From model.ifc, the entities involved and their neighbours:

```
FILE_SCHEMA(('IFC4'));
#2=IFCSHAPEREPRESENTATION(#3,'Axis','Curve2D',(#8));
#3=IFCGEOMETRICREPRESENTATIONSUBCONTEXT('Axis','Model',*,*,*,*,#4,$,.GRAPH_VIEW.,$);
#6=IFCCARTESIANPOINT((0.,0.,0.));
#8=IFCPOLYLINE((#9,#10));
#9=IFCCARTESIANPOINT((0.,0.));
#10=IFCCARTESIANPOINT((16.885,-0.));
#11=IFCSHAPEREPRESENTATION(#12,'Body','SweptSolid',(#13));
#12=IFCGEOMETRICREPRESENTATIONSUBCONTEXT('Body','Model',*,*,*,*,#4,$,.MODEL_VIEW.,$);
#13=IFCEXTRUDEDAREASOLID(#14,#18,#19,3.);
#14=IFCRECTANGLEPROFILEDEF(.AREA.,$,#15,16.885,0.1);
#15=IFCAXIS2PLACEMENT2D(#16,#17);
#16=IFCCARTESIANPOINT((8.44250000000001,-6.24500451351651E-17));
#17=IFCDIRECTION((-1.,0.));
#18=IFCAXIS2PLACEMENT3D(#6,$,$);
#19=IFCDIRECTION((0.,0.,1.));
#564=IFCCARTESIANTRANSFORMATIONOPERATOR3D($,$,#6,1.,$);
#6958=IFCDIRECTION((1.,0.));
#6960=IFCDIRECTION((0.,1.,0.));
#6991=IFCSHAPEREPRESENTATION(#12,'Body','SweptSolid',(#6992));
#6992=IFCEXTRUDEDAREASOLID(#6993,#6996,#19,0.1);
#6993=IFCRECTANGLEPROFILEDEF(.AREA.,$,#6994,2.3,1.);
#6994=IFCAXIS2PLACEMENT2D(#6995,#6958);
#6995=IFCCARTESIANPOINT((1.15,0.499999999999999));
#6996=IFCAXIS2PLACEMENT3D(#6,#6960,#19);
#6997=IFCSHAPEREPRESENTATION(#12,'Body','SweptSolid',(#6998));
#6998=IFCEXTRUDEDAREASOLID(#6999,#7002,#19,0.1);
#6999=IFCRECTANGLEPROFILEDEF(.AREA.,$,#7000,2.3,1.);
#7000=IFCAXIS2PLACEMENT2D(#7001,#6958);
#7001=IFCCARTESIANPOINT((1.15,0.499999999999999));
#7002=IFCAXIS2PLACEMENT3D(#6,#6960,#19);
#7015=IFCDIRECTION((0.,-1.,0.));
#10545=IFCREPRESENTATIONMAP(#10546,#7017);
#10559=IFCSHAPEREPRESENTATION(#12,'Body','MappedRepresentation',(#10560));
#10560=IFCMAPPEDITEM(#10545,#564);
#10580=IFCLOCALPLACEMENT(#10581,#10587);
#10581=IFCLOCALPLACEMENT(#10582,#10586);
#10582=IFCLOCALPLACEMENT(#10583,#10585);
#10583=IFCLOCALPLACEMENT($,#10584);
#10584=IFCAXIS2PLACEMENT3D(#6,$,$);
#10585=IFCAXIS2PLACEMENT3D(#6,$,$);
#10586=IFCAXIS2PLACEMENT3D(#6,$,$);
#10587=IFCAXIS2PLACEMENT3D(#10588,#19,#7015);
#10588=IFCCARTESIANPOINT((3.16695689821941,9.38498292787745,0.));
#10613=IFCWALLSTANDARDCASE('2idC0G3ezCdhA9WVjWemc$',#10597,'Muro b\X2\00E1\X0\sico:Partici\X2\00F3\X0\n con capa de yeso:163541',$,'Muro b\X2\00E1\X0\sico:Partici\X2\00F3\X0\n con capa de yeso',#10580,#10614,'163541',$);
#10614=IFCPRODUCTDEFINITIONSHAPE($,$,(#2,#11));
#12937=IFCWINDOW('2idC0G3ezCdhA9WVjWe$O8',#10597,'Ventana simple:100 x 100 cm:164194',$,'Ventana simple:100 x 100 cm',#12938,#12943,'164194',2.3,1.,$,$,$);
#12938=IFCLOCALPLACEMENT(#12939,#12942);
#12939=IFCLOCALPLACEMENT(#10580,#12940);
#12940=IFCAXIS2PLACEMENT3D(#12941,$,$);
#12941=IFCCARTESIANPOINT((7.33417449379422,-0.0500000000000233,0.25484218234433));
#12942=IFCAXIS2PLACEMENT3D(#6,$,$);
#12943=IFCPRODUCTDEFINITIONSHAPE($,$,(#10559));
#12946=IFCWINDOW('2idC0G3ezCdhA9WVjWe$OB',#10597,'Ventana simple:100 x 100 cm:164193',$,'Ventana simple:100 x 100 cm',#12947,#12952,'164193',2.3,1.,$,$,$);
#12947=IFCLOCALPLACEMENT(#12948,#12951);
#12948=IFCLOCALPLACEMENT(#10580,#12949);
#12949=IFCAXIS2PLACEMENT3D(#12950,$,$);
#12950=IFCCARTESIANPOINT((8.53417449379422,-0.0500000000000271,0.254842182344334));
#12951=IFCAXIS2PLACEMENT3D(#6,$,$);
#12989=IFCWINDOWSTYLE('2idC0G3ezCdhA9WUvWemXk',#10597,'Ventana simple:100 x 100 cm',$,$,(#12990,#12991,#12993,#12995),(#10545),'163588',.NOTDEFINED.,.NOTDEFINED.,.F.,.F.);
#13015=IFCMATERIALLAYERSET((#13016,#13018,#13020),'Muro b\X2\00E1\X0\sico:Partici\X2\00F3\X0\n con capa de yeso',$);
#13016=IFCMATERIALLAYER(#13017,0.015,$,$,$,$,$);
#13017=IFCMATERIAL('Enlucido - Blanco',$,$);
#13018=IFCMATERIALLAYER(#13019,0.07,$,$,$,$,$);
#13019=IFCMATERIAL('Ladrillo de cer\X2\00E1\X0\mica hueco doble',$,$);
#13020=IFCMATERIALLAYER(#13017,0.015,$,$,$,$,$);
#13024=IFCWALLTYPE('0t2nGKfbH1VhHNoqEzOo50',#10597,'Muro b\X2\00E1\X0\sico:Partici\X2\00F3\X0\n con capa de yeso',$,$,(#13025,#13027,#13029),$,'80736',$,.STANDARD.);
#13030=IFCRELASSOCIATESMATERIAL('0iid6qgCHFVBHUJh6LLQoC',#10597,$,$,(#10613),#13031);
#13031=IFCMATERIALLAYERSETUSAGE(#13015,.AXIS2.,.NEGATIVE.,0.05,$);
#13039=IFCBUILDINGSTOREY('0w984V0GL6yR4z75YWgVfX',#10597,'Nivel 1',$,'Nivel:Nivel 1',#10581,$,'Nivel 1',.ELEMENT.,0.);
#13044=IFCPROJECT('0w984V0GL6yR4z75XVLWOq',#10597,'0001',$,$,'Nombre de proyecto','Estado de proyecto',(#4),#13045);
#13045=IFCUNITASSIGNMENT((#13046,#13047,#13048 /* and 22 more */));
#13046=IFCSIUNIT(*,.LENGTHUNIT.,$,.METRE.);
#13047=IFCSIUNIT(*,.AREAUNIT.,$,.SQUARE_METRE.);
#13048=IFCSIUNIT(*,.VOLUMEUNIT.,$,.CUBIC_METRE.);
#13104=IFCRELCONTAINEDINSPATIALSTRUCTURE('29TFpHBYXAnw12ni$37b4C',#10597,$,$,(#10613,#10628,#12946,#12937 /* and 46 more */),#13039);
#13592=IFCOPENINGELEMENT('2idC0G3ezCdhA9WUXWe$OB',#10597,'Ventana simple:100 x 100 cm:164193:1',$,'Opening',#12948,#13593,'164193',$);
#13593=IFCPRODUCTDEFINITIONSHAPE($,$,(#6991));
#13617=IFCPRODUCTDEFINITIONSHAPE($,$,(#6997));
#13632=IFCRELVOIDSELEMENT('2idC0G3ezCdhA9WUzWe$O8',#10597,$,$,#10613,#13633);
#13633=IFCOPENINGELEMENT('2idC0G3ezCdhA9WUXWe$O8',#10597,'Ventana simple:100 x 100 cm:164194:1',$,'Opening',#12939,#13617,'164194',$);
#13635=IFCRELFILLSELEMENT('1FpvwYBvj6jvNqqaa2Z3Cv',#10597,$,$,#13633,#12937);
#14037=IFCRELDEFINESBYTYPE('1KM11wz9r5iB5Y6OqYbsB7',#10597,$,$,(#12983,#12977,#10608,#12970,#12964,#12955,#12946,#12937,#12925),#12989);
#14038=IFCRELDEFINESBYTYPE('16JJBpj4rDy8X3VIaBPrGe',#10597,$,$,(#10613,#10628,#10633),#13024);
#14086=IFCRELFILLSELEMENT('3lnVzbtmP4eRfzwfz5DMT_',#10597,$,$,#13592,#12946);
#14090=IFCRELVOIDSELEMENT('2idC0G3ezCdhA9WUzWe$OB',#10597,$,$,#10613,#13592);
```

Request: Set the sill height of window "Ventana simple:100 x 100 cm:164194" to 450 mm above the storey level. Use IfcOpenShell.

```python
import numpy as np
import ifcopenshell
import ifcopenshell.api.geometry
import ifcopenshell.geom
import ifcopenshell.util.element
import ifcopenshell.util.placement
import ifcopenshell.util.shape
import ifcopenshell.util.unit

model = ifcopenshell.open("model.ifc")
unit_scale = ifcopenshell.util.unit.calculate_unit_scale(model)

window = model.by_id(12937)
opening = window.FillsVoids[0].RelatingOpeningElement
storey = ifcopenshell.util.element.get_container(window, ifc_class="IfcBuildingStorey")
level = ifcopenshell.util.placement.get_local_placement(storey.ObjectPlacement)[2, 3]

# The opening's origin need not be at the sill, so measure its lowest point.
shape = ifcopenshell.geom.create_shape(ifcopenshell.geom.settings(), opening)
bottom = ifcopenshell.util.shape.get_shape_bottom_elevation(shape, shape.geometry) / unit_scale
dz = level + 0.45 / unit_scale - bottom

shift = np.array([0.0, 0.0, dz])
# The window is placed relative to its opening, so it follows when the opening moves.
matrix = ifcopenshell.util.placement.get_local_placement(opening.ObjectPlacement)
matrix[:3, 3] += shift
ifcopenshell.api.geometry.edit_object_placement(
    model, product=opening, matrix=matrix, is_si=False, should_transform_children=True
)

print(f"moved by {dz * unit_scale:+.3f} m")

model.write("model_edited.ifc")
```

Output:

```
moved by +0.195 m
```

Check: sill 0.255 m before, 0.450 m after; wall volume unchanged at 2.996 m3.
